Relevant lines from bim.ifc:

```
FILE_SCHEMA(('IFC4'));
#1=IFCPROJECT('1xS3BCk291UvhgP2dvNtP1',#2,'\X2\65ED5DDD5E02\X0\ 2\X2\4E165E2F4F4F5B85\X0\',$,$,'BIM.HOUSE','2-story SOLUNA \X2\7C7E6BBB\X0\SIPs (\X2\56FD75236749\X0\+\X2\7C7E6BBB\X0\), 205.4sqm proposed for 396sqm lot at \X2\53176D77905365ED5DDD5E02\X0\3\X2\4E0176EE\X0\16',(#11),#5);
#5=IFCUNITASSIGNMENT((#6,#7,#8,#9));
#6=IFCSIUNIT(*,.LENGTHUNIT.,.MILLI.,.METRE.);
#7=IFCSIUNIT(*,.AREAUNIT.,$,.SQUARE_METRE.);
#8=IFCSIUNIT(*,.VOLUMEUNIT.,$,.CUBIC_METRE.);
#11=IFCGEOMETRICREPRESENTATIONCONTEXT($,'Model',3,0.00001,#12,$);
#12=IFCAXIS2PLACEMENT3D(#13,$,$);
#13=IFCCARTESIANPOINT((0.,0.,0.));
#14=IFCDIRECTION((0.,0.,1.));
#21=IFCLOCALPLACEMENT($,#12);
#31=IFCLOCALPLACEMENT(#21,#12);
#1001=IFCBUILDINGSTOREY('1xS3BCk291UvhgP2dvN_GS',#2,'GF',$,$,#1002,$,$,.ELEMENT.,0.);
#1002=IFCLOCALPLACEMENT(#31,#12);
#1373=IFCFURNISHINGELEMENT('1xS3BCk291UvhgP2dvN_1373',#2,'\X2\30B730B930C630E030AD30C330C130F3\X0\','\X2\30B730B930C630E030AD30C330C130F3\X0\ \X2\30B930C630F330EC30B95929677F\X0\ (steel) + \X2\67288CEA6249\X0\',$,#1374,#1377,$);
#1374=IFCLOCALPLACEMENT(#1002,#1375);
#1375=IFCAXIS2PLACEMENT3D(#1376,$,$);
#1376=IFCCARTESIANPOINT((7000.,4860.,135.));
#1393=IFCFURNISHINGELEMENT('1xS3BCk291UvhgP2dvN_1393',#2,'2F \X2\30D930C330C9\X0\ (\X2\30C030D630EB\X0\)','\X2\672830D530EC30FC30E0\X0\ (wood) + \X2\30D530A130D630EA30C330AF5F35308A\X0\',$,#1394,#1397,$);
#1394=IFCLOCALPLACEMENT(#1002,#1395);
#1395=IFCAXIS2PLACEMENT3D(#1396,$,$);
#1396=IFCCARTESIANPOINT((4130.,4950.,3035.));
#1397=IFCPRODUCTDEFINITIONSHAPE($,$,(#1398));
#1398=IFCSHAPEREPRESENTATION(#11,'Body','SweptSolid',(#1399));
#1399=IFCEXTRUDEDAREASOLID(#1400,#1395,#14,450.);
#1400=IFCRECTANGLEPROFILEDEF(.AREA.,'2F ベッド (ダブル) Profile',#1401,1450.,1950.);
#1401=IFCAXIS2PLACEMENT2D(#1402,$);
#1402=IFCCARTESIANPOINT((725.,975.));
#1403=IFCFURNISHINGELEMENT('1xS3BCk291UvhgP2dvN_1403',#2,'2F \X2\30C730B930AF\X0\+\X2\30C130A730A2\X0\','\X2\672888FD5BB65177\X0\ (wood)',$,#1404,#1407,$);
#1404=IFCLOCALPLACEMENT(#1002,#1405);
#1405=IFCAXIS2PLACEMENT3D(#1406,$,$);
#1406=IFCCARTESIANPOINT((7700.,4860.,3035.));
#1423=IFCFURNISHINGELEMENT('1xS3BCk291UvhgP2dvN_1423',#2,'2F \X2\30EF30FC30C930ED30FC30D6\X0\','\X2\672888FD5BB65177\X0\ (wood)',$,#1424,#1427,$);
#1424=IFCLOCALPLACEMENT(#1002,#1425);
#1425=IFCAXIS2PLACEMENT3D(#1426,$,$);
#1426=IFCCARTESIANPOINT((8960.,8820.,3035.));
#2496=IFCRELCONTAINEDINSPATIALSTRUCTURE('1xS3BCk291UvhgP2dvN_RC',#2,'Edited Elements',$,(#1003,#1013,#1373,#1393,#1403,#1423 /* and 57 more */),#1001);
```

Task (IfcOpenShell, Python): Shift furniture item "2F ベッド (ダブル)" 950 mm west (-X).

```python
import ifcopenshell
import ifcopenshell.api.geometry
import ifcopenshell.util.placement

model = ifcopenshell.open("bim.ifc")

item = model.by_guid("1xS3BCk291UvhgP2dvN_1393")
matrix = ifcopenshell.util.placement.get_local_placement(item.ObjectPlacement)
matrix[0, 3] -= 950.0
ifcopenshell.api.geometry.edit_object_placement(model, product=item, matrix=matrix, is_si=False)

print(ifcopenshell.util.placement.get_local_placement(item.ObjectPlacement).round(3) + 0.0)

model.write("bim-out.ifc")
```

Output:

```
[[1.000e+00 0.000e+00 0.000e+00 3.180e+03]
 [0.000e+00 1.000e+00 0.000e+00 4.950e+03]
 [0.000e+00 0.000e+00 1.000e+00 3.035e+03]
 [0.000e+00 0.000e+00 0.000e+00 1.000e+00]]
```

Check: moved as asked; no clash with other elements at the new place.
